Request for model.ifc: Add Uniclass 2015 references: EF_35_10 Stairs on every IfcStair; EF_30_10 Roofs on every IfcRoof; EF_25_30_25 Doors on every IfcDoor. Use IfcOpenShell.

First a look at what the model holds.

```python
import ifcopenshell

model = ifcopenshell.open("model.ifc")
print(model.schema)
print("classifications:", [c.Name for c in model.by_type("IfcClassification")])
for ifc_class in ("IfcDoor", "IfcRoof", "IfcStair", "IfcWall", "IfcWindow"):
    print(ifc_class, len(model.by_type(ifc_class)))
```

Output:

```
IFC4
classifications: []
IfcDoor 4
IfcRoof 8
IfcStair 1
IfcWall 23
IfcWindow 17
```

```python
import ifcopenshell
import ifcopenshell.api.classification

model = ifcopenshell.open("model.ifc")

system = ifcopenshell.api.classification.add_classification(model, classification="Uniclass 2015")

codes = {
    "IfcStair": ("EF_35_10", "Stairs"),
    "IfcRoof": ("EF_30_10", "Roofs"),
    "IfcDoor": ("EF_25_30_25", "Doors"),
}
for ifc_class, (code, name) in codes.items():
    products = model.by_type(ifc_class)
    ifcopenshell.api.classification.add_reference(
        model, products=products, classification=system, identification=code, name=name
    )
    print(code, len(products))

model.write("model_v2.ifc")
```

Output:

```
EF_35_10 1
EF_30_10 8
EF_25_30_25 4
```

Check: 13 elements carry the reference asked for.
